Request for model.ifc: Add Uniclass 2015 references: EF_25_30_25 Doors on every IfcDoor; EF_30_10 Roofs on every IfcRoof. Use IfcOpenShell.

First a look at what the model holds.

```python
import ifcopenshell

model = ifcopenshell.open("model.ifc")
print(model.schema)
print("classifications:", [c.Name for c in model.by_type("IfcClassification")])
for ifc_class in ("IfcDoor", "IfcRoof", "IfcStair", "IfcWall", "IfcWindow"):
    print(ifc_class, len(model.by_type(ifc_class)))
```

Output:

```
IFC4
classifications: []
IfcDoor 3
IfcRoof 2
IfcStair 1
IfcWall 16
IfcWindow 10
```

```python
import ifcopenshell
import ifcopenshell.api.classification

model = ifcopenshell.open("model.ifc")

system = ifcopenshell.api.classification.add_classification(model, classification="Uniclass 2015")

codes = {
    "IfcDoor": ("EF_25_30_25", "Doors"),
    "IfcRoof": ("EF_30_10", "Roofs"),
}
for ifc_class, (code, name) in codes.items():
    products = model.by_type(ifc_class)
    ifcopenshell.api.classification.add_reference(
        model, products=products, classification=system, identification=code, name=name
    )
    print(code, len(products))

model.write("model-out.ifc")
```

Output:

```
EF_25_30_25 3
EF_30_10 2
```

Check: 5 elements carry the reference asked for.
